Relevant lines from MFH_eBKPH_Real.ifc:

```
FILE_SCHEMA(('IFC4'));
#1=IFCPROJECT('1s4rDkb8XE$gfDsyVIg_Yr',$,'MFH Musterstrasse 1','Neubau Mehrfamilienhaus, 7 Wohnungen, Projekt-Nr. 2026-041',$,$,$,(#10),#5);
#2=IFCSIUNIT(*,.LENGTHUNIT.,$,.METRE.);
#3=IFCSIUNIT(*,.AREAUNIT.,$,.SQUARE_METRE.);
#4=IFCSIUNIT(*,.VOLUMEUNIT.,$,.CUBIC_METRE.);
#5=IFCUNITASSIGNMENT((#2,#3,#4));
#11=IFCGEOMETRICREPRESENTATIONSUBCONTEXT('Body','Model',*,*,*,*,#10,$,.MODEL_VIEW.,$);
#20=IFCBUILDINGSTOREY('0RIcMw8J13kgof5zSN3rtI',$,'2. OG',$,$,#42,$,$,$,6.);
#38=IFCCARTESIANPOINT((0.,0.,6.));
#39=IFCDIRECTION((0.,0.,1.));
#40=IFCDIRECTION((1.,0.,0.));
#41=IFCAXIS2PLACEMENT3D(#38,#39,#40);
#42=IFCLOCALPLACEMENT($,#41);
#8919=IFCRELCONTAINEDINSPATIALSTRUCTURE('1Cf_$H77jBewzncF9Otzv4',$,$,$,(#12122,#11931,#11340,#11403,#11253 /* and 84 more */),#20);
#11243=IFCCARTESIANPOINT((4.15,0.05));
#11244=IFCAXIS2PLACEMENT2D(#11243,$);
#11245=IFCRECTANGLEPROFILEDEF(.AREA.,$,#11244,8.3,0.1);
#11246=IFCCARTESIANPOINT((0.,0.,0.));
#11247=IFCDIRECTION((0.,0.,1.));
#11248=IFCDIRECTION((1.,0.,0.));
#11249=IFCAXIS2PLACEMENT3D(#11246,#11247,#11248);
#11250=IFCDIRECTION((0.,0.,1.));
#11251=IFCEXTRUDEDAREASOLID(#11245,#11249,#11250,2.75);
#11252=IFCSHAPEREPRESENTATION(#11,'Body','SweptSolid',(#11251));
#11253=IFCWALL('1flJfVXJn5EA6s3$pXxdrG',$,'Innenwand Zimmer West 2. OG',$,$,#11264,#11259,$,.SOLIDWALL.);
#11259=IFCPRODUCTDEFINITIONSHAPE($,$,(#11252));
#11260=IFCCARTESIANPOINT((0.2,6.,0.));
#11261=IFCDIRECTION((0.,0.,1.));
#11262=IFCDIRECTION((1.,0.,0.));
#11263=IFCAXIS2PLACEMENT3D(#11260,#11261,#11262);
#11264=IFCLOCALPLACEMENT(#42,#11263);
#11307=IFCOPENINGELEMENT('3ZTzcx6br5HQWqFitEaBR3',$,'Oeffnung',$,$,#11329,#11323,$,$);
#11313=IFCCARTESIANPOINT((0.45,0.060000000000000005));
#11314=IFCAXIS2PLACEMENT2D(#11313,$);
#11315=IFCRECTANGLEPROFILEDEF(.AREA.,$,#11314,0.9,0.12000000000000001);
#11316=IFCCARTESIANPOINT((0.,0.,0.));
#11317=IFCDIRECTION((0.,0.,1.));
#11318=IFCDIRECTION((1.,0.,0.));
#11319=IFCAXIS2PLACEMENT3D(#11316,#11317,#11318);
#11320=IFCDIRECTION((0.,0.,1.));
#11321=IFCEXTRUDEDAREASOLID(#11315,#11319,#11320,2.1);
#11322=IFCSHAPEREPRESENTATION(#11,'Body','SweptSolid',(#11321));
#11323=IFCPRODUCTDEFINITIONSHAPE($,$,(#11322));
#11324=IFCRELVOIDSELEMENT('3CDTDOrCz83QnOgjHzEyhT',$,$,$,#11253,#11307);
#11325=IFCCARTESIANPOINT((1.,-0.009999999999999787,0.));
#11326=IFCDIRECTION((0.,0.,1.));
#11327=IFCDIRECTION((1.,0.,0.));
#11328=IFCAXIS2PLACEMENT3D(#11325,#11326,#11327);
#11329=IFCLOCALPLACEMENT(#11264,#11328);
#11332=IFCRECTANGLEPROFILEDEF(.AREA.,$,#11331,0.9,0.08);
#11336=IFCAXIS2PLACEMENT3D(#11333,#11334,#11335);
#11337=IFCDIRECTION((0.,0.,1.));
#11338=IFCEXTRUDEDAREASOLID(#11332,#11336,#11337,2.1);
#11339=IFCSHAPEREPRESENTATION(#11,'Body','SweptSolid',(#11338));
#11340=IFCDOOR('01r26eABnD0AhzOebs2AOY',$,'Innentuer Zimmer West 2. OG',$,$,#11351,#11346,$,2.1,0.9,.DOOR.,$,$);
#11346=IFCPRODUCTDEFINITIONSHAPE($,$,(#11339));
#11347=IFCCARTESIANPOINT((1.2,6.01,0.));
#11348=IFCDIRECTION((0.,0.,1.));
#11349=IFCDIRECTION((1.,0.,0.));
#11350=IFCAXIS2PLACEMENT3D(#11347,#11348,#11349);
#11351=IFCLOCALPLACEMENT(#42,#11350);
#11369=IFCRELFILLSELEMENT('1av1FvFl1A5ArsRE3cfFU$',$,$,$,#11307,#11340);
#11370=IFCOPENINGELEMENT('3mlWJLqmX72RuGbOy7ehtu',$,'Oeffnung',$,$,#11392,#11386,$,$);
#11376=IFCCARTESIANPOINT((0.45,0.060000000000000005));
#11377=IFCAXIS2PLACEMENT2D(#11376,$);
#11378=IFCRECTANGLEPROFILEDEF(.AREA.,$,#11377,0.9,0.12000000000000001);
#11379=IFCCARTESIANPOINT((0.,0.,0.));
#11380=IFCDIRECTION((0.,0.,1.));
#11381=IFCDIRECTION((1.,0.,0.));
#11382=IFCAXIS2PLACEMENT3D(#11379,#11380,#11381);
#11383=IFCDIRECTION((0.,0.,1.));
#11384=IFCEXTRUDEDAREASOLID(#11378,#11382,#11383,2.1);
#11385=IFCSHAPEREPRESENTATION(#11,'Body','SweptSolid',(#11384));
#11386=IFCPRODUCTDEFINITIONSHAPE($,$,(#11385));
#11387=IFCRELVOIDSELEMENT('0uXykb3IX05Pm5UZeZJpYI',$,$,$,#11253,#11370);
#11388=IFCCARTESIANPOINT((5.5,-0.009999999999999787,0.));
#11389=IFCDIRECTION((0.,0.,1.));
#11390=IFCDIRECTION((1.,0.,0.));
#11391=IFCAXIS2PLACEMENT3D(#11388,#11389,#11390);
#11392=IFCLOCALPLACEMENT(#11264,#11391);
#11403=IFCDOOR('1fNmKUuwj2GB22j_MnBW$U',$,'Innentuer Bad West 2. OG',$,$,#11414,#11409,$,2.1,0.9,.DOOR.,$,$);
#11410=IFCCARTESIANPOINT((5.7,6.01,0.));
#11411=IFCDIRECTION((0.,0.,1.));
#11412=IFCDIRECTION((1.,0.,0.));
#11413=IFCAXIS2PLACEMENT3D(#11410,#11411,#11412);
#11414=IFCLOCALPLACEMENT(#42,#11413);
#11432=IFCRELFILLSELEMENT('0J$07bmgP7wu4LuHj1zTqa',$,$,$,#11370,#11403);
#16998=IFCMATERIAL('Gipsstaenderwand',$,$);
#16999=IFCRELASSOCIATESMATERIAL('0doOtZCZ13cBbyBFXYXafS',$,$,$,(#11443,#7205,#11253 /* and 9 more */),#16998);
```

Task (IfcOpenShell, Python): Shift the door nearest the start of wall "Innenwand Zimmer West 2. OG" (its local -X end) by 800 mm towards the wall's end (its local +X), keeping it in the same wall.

```python
import ifcopenshell
import ifcopenshell.api.geometry
import ifcopenshell.util.placement
import ifcopenshell.util.unit

model = ifcopenshell.open("MFH_eBKPH_Real.ifc")
unit_scale = ifcopenshell.util.unit.calculate_unit_scale(model)

door = model.by_guid("01r26eABnD0AhzOebs2AOY")
opening = door.FillsVoids[0].RelatingOpeningElement
wall = opening.VoidsElements[0].RelatingBuildingElement

wall_matrix = ifcopenshell.util.placement.get_local_placement(wall.ObjectPlacement)
shift = wall_matrix[:3, 0] * 0.8 / unit_scale
before = ifcopenshell.util.placement.get_local_placement(door.ObjectPlacement)[:3, 3].copy()

# The door is not placed relative to its opening, so move both.
for product in (opening, door):
    matrix = ifcopenshell.util.placement.get_local_placement(product.ObjectPlacement)
    matrix[:3, 3] += shift
    ifcopenshell.api.geometry.edit_object_placement(model, product=product, matrix=matrix, is_si=False)

after = ifcopenshell.util.placement.get_local_placement(door.ObjectPlacement)[:3, 3]
print("door moved by", (after - before).round(3) + 0.0)

model.write("MFH_eBKPH_Real_updated.ifc")
```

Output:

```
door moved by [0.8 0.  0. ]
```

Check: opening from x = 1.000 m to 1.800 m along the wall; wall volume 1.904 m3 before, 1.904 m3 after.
